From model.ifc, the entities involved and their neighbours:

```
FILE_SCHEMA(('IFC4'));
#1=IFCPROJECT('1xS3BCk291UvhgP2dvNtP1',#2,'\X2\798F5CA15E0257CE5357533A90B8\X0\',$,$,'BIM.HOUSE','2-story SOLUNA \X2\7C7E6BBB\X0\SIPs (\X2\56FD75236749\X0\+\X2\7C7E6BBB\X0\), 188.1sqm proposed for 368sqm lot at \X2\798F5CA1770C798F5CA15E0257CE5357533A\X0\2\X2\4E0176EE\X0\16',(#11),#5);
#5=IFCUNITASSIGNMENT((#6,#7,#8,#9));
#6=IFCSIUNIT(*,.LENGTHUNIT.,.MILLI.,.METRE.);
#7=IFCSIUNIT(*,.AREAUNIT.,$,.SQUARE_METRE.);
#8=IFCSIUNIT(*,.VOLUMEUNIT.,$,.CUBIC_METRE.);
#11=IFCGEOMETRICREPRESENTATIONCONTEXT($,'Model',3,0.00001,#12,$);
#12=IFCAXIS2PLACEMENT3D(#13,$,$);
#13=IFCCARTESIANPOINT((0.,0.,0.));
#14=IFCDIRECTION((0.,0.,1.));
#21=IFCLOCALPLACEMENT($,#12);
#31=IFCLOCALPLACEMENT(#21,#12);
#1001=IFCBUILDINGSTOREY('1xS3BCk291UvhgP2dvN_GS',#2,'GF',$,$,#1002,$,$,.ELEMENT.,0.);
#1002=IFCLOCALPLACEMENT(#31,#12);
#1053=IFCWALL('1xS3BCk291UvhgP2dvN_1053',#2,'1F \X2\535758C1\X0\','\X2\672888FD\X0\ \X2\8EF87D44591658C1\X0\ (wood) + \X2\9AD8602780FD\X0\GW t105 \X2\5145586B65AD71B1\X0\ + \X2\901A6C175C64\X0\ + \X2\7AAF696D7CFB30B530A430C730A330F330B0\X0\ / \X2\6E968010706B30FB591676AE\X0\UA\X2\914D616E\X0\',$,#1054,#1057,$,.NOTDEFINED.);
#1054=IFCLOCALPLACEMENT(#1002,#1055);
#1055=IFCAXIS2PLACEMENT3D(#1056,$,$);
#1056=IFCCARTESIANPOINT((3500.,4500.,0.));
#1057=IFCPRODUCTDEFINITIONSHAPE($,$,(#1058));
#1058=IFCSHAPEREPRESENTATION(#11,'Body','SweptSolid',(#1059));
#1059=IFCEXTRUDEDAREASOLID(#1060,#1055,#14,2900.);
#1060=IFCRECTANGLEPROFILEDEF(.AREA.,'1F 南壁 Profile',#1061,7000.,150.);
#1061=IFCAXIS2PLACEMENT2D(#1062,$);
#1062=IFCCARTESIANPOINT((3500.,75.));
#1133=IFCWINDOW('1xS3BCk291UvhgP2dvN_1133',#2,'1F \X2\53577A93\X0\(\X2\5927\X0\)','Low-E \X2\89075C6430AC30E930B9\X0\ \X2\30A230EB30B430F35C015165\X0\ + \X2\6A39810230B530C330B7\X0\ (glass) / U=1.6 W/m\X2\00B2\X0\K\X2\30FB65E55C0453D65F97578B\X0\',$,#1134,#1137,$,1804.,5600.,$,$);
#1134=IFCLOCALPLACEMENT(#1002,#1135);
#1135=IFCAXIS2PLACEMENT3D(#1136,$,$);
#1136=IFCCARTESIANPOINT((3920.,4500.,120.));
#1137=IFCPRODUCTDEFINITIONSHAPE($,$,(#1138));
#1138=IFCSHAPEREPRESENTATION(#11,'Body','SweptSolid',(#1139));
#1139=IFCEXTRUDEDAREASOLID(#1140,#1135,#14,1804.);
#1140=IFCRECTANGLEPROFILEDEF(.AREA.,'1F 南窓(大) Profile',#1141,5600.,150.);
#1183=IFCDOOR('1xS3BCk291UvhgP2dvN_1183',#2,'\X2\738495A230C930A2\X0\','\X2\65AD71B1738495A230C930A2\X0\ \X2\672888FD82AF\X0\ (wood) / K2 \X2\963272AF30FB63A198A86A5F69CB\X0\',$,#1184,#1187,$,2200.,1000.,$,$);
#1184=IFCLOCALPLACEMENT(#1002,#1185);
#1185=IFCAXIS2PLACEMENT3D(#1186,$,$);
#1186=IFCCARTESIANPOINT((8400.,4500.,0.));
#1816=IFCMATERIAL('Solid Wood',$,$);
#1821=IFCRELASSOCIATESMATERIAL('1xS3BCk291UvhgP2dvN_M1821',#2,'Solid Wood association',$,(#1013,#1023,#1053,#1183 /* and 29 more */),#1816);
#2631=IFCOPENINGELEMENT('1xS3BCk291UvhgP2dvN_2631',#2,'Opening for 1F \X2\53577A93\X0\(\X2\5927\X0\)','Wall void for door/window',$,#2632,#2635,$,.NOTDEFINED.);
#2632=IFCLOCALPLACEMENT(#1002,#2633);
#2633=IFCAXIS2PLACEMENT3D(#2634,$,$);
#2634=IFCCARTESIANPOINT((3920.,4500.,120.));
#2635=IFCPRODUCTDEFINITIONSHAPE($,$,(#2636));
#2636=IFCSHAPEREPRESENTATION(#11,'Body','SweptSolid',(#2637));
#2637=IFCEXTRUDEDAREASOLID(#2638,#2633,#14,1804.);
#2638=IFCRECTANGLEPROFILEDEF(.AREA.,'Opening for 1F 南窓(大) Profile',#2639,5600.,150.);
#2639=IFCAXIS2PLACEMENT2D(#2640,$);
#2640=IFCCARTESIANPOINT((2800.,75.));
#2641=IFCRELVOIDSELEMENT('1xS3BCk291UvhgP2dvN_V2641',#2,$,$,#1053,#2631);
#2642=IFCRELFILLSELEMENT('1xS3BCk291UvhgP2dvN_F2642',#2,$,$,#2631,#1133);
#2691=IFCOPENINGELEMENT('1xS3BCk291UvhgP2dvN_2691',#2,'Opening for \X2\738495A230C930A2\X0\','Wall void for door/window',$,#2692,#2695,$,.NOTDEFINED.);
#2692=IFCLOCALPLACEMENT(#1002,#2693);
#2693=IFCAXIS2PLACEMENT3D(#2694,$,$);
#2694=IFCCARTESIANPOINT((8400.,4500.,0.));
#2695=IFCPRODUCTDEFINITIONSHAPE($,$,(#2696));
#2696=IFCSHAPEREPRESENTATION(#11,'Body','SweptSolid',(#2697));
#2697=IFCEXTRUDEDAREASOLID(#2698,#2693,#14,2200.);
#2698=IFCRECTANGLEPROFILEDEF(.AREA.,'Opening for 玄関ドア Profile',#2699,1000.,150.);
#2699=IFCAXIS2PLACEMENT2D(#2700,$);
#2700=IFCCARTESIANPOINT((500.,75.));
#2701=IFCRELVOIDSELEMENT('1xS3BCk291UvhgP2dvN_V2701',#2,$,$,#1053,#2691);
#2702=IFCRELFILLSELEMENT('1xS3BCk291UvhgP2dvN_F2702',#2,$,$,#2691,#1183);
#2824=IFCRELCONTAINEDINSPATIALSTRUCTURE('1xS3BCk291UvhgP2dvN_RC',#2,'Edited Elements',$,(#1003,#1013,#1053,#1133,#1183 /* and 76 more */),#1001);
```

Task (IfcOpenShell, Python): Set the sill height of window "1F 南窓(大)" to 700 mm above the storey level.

```python
import numpy as np
import ifcopenshell
import ifcopenshell.api.geometry
import ifcopenshell.geom
import ifcopenshell.util.element
import ifcopenshell.util.placement
import ifcopenshell.util.shape
import ifcopenshell.util.unit

model = ifcopenshell.open("model.ifc")
unit_scale = ifcopenshell.util.unit.calculate_unit_scale(model)

window = model.by_id(1133)
opening = window.FillsVoids[0].RelatingOpeningElement
storey = ifcopenshell.util.element.get_container(window, ifc_class="IfcBuildingStorey")
level = ifcopenshell.util.placement.get_local_placement(storey.ObjectPlacement)[2, 3]

# The opening's origin need not be at the sill, so measure its lowest point.
shape = ifcopenshell.geom.create_shape(ifcopenshell.geom.settings(), opening)
bottom = ifcopenshell.util.shape.get_shape_bottom_elevation(shape, shape.geometry) / unit_scale
dz = level + 700.0 - bottom

shift = np.array([0.0, 0.0, dz])
# The window is not placed relative to its opening, so move both.
for product in (opening, window):
    matrix = ifcopenshell.util.placement.get_local_placement(product.ObjectPlacement)
    matrix[:3, 3] += shift
    ifcopenshell.api.geometry.edit_object_placement(model, product=product, matrix=matrix, is_si=False)

print(f"moved by {dz * unit_scale:+.3f} m")

model.write("model_rev.ifc")
```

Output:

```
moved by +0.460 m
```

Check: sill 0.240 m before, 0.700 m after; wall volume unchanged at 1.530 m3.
